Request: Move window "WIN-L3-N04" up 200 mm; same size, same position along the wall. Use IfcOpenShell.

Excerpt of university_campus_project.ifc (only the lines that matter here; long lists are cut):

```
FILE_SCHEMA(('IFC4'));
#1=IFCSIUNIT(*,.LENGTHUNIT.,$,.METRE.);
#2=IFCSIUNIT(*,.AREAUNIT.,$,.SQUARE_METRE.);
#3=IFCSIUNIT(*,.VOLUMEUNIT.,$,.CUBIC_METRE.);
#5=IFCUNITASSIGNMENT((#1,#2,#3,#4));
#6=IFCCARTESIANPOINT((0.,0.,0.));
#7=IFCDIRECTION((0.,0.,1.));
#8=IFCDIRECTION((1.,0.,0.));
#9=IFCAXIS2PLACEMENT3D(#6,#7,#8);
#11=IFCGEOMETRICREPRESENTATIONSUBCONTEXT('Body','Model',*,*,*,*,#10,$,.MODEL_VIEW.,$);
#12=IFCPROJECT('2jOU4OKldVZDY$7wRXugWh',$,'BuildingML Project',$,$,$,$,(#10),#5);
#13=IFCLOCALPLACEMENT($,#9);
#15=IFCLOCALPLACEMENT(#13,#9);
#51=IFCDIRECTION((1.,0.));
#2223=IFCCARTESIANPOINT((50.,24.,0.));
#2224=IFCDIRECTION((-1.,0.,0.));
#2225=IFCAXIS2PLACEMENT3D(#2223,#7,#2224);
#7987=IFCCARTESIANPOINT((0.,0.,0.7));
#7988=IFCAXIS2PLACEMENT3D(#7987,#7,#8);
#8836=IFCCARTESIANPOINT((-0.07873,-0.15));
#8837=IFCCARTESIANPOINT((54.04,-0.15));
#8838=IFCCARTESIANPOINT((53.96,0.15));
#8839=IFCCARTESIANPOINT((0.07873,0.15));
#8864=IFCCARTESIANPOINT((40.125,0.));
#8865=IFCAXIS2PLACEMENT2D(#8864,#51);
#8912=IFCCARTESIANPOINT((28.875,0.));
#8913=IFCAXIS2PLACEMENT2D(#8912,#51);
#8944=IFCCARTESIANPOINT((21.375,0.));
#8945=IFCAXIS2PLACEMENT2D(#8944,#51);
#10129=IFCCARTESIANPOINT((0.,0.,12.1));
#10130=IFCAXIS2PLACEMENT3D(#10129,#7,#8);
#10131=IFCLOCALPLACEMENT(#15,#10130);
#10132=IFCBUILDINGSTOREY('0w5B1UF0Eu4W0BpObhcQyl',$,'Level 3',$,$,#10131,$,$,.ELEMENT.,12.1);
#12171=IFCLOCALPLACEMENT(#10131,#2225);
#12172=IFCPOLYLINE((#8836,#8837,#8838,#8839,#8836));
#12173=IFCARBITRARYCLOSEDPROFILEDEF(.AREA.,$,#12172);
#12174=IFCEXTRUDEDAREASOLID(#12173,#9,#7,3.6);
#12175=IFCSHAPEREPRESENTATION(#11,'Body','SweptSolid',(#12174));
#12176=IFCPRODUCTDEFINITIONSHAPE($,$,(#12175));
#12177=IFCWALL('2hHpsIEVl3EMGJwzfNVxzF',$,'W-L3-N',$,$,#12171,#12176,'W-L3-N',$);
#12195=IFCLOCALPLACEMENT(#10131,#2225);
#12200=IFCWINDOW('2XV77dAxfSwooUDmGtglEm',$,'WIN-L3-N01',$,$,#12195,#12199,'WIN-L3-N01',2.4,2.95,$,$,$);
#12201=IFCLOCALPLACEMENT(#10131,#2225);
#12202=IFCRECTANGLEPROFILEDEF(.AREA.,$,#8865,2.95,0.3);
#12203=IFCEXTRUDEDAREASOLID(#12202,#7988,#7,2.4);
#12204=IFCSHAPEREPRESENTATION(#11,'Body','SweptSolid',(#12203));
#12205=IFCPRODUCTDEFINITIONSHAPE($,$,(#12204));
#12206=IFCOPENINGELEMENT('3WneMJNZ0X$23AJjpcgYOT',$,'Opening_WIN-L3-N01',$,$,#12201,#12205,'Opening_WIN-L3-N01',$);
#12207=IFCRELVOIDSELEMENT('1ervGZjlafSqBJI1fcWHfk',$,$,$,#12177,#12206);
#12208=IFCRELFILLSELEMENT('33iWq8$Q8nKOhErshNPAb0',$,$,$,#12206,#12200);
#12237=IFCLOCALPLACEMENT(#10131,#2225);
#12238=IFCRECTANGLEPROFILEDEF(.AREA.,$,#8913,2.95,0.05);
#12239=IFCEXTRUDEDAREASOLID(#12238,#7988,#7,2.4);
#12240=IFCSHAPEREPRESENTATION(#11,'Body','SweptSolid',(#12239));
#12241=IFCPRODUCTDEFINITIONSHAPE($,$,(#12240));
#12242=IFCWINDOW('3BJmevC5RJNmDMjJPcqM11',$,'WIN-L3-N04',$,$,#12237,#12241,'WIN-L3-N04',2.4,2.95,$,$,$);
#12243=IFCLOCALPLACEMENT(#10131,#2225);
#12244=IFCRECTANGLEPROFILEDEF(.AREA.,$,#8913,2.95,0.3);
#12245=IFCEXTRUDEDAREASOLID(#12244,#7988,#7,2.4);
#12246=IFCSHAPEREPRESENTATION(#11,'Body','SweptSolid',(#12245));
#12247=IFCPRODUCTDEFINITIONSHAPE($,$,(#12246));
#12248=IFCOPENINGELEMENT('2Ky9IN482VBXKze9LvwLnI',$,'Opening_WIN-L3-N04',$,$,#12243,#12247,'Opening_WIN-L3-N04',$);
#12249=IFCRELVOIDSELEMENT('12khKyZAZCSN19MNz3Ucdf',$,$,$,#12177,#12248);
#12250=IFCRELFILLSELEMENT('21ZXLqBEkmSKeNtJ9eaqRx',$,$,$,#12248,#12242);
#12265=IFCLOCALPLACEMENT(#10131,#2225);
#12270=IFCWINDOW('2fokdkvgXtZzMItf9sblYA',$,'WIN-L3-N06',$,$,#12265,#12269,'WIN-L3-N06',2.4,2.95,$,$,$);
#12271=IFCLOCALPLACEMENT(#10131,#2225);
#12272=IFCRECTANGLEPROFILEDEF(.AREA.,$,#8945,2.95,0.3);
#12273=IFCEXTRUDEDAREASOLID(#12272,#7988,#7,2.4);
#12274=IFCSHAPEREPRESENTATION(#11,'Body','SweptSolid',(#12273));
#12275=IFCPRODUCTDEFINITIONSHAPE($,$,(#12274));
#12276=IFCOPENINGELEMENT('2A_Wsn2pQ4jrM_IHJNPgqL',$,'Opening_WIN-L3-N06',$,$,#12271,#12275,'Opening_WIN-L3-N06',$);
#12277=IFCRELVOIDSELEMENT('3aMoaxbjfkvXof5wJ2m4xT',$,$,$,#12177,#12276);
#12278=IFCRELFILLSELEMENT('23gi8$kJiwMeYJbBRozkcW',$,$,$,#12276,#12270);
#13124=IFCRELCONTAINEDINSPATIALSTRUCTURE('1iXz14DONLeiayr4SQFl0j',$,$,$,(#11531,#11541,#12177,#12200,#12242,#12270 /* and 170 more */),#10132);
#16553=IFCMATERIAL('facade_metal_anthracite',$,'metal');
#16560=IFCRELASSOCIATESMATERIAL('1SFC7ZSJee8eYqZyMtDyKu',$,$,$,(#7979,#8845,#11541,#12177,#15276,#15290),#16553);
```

```python
import numpy as np
import ifcopenshell
import ifcopenshell.api.geometry
import ifcopenshell.util.placement
import ifcopenshell.util.unit

model = ifcopenshell.open("university_campus_project.ifc")
unit_scale = ifcopenshell.util.unit.calculate_unit_scale(model)

window = model.by_id(12242)
opening = window.FillsVoids[0].RelatingOpeningElement
dz = 0.2

shift = np.array([0.0, 0.0, dz])
# The window is not placed relative to its opening, so move both.
for product in (opening, window):
    matrix = ifcopenshell.util.placement.get_local_placement(product.ObjectPlacement)
    matrix[:3, 3] += shift
    ifcopenshell.api.geometry.edit_object_placement(model, product=product, matrix=matrix, is_si=False)

print(f"moved by {dz * unit_scale:+.3f} m")

model.write("university_campus_project_updated.ifc")
```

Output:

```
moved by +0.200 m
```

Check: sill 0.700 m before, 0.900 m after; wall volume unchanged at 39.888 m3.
